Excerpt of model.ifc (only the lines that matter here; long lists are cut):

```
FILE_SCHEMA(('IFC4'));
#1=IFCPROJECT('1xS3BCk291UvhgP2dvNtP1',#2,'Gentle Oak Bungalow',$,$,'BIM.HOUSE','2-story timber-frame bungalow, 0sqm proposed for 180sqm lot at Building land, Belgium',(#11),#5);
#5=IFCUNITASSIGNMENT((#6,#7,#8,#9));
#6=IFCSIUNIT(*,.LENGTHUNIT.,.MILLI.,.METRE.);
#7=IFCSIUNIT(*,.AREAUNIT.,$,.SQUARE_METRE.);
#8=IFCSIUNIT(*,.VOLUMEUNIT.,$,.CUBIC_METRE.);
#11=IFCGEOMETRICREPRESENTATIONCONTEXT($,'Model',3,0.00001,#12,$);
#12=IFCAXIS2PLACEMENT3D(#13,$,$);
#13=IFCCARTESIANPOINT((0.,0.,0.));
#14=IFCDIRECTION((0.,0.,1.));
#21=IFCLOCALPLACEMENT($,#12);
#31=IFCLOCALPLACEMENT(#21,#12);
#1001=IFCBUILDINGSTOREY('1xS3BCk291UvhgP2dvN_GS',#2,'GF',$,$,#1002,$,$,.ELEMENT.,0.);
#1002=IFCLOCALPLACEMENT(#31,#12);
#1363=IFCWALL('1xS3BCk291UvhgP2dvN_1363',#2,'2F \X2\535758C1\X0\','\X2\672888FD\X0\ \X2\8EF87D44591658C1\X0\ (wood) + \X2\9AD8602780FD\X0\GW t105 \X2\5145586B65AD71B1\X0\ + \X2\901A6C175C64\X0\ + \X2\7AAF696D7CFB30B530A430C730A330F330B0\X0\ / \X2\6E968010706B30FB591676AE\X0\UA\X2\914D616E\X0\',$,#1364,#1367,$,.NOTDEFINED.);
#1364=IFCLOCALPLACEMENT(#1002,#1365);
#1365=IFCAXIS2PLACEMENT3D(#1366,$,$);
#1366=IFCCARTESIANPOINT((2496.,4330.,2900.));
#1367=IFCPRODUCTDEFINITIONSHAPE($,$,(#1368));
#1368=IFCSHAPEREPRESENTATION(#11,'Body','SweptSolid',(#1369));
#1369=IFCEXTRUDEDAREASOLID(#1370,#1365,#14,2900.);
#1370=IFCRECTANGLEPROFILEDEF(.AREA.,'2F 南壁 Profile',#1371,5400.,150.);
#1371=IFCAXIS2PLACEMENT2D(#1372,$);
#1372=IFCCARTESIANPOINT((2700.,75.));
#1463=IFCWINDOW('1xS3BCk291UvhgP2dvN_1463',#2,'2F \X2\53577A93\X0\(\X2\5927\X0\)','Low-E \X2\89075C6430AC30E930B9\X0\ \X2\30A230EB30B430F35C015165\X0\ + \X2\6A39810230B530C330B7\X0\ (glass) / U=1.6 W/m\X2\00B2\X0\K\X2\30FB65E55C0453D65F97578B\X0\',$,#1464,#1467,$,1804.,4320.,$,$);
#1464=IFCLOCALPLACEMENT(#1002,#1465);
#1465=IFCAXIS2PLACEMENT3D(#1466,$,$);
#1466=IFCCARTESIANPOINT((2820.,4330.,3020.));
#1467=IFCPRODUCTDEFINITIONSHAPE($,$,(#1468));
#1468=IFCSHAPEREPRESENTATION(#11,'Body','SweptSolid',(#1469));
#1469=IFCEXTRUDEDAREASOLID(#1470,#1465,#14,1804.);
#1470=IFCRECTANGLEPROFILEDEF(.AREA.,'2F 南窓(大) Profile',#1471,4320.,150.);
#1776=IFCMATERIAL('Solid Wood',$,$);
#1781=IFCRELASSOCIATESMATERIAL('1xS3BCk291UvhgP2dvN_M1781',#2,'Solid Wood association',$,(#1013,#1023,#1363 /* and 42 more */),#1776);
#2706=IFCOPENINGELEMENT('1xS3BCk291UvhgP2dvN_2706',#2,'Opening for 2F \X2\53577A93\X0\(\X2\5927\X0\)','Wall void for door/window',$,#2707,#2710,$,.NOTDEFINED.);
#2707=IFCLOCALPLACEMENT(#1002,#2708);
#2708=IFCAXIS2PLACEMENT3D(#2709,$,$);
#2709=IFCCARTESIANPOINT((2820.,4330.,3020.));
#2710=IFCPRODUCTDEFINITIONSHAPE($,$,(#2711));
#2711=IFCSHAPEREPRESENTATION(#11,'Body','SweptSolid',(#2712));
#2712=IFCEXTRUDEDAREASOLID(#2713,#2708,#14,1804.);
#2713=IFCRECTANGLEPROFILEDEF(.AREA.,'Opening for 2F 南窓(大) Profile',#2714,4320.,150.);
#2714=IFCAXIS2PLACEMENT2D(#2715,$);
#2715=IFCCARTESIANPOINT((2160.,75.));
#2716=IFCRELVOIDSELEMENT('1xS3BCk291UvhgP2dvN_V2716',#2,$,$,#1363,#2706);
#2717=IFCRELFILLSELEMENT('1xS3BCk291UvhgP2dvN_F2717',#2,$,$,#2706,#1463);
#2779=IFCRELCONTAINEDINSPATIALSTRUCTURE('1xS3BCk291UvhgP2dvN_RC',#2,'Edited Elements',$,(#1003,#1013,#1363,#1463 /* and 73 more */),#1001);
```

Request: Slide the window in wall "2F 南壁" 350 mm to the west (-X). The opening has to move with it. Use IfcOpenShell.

```python
import ifcopenshell
import ifcopenshell.api.geometry
import ifcopenshell.util.placement
import ifcopenshell.util.unit

model = ifcopenshell.open("model.ifc")
unit_scale = ifcopenshell.util.unit.calculate_unit_scale(model)

window = model.by_guid("1xS3BCk291UvhgP2dvN_1463")
opening = window.FillsVoids[0].RelatingOpeningElement
wall = opening.VoidsElements[0].RelatingBuildingElement

wall_matrix = ifcopenshell.util.placement.get_local_placement(wall.ObjectPlacement)
shift = wall_matrix[:3, 0] * -0.35 / unit_scale
before = ifcopenshell.util.placement.get_local_placement(window.ObjectPlacement)[:3, 3].copy()

# The window is not placed relative to its opening, so move both.
for product in (opening, window):
    matrix = ifcopenshell.util.placement.get_local_placement(product.ObjectPlacement)
    matrix[:3, 3] += shift
    ifcopenshell.api.geometry.edit_object_placement(model, product=product, matrix=matrix, is_si=False)

after = ifcopenshell.util.placement.get_local_placement(window.ObjectPlacement)[:3, 3]
print("window moved by", (after - before).round(3) + 0.0)

model.write("model_rev.ifc")
```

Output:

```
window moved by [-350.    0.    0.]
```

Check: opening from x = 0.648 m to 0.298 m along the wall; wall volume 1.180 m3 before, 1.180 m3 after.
